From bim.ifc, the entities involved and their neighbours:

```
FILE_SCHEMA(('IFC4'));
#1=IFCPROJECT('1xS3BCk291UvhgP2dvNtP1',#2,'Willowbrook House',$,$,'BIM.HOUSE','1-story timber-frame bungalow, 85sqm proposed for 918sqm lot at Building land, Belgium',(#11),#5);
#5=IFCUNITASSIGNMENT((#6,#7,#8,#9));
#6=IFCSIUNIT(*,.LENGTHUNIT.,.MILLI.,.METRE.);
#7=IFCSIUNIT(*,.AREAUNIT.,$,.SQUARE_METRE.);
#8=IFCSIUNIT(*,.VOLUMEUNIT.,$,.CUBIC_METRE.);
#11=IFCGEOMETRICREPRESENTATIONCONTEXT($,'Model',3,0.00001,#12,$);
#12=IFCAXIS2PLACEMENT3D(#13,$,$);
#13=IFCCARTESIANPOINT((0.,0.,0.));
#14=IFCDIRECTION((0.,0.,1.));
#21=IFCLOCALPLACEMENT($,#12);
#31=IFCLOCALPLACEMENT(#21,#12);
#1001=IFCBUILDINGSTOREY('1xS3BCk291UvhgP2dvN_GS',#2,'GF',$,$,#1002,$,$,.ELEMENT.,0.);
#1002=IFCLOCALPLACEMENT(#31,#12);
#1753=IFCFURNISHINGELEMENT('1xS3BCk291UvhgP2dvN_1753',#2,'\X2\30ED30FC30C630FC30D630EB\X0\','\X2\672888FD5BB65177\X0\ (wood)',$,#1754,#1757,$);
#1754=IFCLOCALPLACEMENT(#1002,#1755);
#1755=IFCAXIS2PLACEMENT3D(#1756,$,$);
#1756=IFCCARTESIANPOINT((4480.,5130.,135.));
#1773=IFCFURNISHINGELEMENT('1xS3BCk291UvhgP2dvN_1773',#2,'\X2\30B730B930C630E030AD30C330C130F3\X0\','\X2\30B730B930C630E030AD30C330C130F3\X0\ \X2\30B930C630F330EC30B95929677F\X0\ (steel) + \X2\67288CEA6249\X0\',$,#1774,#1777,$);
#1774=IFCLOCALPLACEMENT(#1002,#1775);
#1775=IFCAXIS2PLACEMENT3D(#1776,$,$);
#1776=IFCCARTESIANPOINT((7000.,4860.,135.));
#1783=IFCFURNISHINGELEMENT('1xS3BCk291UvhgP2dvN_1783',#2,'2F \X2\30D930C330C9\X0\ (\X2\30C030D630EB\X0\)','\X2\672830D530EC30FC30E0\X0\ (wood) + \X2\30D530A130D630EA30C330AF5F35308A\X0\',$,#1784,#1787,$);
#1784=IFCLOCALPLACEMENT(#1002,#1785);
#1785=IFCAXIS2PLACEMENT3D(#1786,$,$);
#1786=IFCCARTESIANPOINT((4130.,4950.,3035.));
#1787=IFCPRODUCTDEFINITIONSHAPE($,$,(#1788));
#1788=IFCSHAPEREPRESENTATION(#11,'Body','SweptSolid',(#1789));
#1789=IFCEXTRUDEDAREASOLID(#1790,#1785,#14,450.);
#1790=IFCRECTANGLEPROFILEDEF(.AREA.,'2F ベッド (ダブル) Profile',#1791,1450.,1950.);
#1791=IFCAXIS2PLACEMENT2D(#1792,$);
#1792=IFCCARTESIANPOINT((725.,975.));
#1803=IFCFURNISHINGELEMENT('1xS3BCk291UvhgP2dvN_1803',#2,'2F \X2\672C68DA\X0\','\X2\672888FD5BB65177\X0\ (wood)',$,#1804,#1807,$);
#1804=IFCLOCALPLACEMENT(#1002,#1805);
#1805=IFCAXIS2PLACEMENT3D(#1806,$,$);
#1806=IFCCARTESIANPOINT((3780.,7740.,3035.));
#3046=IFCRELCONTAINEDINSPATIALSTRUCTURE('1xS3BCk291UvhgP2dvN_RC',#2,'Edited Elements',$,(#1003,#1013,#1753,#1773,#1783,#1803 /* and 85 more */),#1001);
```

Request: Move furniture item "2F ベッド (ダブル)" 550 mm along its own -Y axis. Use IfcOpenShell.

```python
import ifcopenshell
import ifcopenshell.api.geometry
import ifcopenshell.util.placement
import ifcopenshell.util.unit

model = ifcopenshell.open("bim.ifc")
unit_scale = ifcopenshell.util.unit.calculate_unit_scale(model)

item = model.by_id(1783)
matrix = ifcopenshell.util.placement.get_local_placement(item.ObjectPlacement)
matrix[:3, 3] -= matrix[:3, 1] * 0.55 / unit_scale
ifcopenshell.api.geometry.edit_object_placement(model, product=item, matrix=matrix, is_si=False)

print(ifcopenshell.util.placement.get_local_placement(item.ObjectPlacement).round(3) + 0.0)

model.write("bim-out.ifc")
```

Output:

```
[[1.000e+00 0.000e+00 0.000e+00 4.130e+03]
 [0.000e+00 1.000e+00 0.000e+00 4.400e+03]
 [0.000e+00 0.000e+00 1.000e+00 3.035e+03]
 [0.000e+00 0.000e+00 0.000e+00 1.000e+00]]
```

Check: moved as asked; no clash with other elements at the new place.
